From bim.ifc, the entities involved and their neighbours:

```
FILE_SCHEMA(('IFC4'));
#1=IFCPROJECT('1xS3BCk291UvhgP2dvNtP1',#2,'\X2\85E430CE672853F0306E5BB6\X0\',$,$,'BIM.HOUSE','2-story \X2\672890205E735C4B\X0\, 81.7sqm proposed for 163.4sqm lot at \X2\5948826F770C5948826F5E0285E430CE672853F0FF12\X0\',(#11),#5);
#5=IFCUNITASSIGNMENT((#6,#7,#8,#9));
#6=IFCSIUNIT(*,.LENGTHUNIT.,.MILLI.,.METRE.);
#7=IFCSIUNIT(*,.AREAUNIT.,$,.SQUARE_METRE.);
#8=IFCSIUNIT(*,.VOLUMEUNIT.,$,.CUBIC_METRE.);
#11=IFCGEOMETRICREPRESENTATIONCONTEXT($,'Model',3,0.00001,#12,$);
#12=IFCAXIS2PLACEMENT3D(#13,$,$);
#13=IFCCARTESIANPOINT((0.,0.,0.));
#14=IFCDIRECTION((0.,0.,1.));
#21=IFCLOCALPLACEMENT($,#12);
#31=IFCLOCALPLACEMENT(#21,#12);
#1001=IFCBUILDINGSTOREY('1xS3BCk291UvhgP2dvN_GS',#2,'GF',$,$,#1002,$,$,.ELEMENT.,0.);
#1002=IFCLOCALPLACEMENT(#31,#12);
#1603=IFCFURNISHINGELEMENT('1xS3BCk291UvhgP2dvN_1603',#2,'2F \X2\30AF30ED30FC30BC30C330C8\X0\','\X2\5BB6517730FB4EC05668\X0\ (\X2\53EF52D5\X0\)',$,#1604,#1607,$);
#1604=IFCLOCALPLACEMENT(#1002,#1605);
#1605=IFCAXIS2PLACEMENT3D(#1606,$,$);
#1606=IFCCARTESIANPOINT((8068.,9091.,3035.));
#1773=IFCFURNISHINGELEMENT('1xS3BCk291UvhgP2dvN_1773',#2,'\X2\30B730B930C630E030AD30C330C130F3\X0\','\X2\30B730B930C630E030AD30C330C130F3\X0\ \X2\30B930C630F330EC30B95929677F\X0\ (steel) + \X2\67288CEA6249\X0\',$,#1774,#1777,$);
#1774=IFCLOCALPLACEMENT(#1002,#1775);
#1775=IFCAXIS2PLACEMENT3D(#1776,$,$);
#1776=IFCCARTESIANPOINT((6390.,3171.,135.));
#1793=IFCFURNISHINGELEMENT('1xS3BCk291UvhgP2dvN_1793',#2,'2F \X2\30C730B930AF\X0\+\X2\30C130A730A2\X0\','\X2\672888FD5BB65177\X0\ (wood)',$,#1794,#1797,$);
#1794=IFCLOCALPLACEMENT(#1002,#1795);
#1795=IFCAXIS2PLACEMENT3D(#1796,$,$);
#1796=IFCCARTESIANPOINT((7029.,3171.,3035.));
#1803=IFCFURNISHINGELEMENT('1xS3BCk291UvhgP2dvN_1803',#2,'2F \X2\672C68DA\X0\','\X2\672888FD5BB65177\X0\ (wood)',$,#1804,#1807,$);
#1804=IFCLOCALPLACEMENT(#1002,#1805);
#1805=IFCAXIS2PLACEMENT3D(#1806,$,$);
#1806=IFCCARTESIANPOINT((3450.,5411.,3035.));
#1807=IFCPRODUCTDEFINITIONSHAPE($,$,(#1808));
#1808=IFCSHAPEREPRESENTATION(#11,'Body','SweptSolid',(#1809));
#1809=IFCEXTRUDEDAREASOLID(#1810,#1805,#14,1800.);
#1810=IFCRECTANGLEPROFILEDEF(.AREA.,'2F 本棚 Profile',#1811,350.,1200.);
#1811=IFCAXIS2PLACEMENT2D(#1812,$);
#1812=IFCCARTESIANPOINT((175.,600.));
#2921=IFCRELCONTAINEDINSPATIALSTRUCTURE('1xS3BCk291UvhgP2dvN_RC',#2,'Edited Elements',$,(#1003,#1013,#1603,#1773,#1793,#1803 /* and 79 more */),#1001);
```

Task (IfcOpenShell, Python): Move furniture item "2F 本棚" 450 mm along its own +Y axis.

```python
import ifcopenshell
import ifcopenshell.api.geometry
import ifcopenshell.util.placement
import ifcopenshell.util.unit

model = ifcopenshell.open("bim.ifc")
unit_scale = ifcopenshell.util.unit.calculate_unit_scale(model)

item = model.by_guid("1xS3BCk291UvhgP2dvN_1803")
matrix = ifcopenshell.util.placement.get_local_placement(item.ObjectPlacement)
matrix[:3, 3] += matrix[:3, 1] * 0.45 / unit_scale
ifcopenshell.api.geometry.edit_object_placement(model, product=item, matrix=matrix, is_si=False)

print(ifcopenshell.util.placement.get_local_placement(item.ObjectPlacement).round(3) + 0.0)

model.write("bim-out.ifc")
```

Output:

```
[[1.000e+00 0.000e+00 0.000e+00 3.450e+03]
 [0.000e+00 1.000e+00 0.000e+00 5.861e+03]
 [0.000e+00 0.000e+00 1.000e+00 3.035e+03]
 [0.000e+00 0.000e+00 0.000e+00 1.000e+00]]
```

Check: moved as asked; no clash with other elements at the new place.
